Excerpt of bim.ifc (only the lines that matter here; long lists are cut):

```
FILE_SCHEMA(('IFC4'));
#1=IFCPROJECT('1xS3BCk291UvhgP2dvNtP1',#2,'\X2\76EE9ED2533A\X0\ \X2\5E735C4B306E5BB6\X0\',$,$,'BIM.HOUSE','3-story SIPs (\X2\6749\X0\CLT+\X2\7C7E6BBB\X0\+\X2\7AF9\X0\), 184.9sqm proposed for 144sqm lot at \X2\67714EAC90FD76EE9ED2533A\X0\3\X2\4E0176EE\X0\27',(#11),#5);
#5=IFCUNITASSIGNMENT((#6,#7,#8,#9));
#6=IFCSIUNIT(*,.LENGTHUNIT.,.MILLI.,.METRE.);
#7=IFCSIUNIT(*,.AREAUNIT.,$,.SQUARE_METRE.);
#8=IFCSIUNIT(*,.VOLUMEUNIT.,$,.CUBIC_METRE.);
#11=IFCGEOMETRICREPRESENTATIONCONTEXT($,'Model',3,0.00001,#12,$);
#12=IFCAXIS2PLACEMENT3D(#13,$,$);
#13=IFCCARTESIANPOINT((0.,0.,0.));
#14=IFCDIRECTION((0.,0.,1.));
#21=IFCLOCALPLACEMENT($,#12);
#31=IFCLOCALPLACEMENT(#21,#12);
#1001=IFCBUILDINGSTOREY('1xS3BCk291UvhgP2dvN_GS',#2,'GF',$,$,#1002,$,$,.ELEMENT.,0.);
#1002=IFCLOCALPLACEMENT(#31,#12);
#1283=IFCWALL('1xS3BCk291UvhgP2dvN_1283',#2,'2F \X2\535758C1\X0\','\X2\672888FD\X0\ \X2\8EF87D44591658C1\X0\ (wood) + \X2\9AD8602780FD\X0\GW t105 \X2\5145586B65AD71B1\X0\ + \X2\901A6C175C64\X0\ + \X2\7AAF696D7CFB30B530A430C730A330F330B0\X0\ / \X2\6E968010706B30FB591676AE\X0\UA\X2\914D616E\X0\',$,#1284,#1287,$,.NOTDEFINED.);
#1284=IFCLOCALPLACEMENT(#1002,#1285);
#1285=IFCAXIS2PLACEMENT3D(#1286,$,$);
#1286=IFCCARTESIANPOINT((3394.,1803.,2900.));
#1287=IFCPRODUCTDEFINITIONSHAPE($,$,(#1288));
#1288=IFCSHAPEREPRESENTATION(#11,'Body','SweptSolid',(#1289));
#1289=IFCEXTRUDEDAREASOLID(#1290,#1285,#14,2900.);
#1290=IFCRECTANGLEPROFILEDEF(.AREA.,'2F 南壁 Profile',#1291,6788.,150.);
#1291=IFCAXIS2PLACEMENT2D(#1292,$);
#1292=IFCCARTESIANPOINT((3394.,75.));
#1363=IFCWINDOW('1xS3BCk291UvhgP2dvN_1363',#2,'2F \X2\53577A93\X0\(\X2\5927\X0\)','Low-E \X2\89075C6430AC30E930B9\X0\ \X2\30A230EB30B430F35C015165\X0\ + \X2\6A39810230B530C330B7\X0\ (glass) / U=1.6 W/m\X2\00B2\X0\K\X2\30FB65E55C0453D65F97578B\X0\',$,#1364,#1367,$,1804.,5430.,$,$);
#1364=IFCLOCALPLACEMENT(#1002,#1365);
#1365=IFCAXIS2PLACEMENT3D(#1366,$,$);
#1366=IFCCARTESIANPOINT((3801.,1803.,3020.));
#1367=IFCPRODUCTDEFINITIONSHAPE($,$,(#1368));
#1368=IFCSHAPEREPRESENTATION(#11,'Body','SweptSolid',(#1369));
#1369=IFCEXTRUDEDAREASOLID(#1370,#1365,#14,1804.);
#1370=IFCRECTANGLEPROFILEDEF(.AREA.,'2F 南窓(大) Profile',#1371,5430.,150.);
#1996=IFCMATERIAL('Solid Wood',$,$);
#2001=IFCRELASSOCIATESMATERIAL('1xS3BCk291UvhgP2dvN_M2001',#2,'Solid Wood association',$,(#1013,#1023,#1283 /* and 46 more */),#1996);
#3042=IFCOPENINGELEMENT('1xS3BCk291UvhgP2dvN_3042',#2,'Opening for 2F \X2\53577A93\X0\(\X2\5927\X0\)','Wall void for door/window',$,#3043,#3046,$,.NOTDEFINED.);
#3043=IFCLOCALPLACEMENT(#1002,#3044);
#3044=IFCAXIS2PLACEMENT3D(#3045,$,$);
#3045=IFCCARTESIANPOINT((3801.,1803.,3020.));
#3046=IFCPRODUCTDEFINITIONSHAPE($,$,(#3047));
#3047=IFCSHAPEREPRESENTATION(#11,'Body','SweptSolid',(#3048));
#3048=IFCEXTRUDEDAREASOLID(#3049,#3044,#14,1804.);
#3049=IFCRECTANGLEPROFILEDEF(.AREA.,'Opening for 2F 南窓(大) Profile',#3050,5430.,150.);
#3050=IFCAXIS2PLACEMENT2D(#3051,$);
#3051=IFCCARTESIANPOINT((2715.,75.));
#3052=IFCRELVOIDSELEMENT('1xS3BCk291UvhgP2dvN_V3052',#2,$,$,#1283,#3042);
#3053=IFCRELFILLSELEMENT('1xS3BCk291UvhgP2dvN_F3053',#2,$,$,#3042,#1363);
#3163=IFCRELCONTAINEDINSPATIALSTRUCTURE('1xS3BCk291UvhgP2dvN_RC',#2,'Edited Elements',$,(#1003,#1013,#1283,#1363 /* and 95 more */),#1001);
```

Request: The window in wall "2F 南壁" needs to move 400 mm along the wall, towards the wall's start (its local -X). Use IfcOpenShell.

```python
import ifcopenshell
import ifcopenshell.api.geometry
import ifcopenshell.util.placement

model = ifcopenshell.open("bim.ifc")

window = model.by_guid("1xS3BCk291UvhgP2dvN_1363")
opening = window.FillsVoids[0].RelatingOpeningElement
wall = opening.VoidsElements[0].RelatingBuildingElement

wall_matrix = ifcopenshell.util.placement.get_local_placement(wall.ObjectPlacement)
shift = wall_matrix[:3, 0] * -400.0
before = ifcopenshell.util.placement.get_local_placement(window.ObjectPlacement)[:3, 3].copy()

# The window is not placed relative to its opening, so move both.
for product in (opening, window):
    matrix = ifcopenshell.util.placement.get_local_placement(product.ObjectPlacement)
    matrix[:3, 3] += shift
    ifcopenshell.api.geometry.edit_object_placement(model, product=product, matrix=matrix, is_si=False)

after = ifcopenshell.util.placement.get_local_placement(window.ObjectPlacement)[:3, 3]
print("window moved by", (after - before).round(3) + 0.0)

model.write("bim_v2.ifc")
```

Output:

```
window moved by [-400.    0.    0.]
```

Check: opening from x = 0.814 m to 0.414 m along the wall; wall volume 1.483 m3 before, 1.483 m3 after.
